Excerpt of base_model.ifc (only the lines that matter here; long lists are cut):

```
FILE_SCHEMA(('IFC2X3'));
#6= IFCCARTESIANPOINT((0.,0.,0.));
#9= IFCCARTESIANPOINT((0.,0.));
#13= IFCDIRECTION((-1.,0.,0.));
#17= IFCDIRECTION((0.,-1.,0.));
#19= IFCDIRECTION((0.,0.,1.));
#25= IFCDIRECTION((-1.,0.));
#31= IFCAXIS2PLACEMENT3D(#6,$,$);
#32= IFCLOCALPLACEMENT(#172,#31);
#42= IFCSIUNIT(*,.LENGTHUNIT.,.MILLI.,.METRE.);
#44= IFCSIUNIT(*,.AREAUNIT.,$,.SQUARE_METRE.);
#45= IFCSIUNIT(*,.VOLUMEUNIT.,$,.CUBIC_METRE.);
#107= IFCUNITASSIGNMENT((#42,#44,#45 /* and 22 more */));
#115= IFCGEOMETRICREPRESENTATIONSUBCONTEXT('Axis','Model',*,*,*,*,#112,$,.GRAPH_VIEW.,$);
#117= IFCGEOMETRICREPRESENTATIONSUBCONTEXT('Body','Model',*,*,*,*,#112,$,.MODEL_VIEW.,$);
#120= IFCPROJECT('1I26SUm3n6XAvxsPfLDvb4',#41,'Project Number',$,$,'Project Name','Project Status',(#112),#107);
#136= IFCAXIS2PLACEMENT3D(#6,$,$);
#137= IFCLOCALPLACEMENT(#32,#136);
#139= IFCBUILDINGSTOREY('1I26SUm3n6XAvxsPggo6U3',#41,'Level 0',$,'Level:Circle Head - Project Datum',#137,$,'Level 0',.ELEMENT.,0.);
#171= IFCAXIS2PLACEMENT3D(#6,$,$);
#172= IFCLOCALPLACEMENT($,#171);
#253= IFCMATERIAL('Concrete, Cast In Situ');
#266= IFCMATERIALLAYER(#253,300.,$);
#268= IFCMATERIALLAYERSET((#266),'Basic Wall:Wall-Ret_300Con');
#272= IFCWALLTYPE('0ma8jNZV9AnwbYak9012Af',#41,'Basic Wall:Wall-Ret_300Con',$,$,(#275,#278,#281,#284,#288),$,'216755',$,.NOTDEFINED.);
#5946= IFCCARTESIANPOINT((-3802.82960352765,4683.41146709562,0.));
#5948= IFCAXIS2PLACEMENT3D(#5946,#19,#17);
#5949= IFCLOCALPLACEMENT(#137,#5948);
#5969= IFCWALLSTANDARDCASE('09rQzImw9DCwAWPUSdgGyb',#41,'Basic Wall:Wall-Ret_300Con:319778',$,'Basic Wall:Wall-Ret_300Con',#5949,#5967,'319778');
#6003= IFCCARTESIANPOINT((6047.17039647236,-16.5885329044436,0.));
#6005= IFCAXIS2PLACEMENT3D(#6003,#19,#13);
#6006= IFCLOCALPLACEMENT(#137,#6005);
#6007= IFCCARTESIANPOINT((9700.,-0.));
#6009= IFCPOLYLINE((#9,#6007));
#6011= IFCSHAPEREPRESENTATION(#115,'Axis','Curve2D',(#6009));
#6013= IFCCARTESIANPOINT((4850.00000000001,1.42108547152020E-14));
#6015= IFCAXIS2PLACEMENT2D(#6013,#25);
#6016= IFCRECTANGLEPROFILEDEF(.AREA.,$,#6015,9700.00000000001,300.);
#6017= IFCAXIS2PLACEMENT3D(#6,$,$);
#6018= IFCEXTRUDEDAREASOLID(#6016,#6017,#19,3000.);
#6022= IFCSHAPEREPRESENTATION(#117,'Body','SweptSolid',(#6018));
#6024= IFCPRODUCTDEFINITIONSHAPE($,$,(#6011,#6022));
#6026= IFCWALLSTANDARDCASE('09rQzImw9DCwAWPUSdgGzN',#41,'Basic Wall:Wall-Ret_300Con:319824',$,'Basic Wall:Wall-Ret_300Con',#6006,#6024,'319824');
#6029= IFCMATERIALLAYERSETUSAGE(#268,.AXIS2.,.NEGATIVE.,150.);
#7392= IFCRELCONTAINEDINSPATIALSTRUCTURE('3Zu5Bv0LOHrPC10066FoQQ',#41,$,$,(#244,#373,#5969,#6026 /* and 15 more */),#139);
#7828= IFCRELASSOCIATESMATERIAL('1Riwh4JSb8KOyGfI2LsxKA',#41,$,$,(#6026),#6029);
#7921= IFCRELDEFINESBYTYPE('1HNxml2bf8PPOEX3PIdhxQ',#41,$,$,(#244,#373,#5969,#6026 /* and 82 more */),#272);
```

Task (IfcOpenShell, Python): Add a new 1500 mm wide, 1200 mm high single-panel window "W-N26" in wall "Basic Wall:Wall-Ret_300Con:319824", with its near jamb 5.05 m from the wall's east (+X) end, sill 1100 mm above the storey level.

```python
import numpy as np
import ifcopenshell
import ifcopenshell.api.feature
import ifcopenshell.api.geometry
import ifcopenshell.api.root
import ifcopenshell.api.spatial
import ifcopenshell.api.type
import ifcopenshell.geom
import ifcopenshell.util.element
import ifcopenshell.util.placement
import ifcopenshell.util.representation
import ifcopenshell.util.shape
import ifcopenshell.util.unit

model = ifcopenshell.open("base_model.ifc")
unit_scale = ifcopenshell.util.unit.calculate_unit_scale(model)
settings = ifcopenshell.geom.settings()


def volume(element):
    """Net volume in cubic metres, openings subtracted."""
    shape = ifcopenshell.geom.create_shape(settings, element)
    return ifcopenshell.util.shape.get_volume(shape.geometry)


wall = model.by_id(6026)
storey = ifcopenshell.util.element.get_container(wall, ifc_class="IfcBuildingStorey")
context = ifcopenshell.util.representation.get_context(model, "Model", "Body", "MODEL_VIEW")
before = volume(wall)

width, height, from_end, sill = 1.5, 1.2, 5.05, 1.1  # metres

# The wall runs along its own X axis, and the end named is its -X end.
wall_shape = ifcopenshell.geom.create_shape(settings, wall)
x, y, z = ifcopenshell.util.shape.get_vertices(wall_shape.geometry).T
start = x.min() + from_end
face, thickness = float(y.min()), float(y.max() - y.min())
wall_matrix = ifcopenshell.util.placement.get_local_placement(wall.ObjectPlacement)
level = ifcopenshell.util.placement.get_local_placement(storey.ObjectPlacement)[2, 3]


def in_wall(x, y):
    """Placement at x, y metres in the wall's axes, at sill height."""
    matrix = wall_matrix.copy()
    matrix[:, 3] = wall_matrix @ np.array([x / unit_scale, y / unit_scale, 0.0, 1.0])
    matrix[2, 3] = level + sill / unit_scale
    return matrix


# Opening: a box that overshoots both wall faces by 50 mm.
opening = ifcopenshell.api.root.create_entity(model, ifc_class="IfcOpeningElement")
box = ifcopenshell.api.geometry.add_wall_representation(
    model, context=context, length=width, height=height, thickness=thickness + 0.1
)
ifcopenshell.api.geometry.assign_representation(model, product=opening, representation=box)
ifcopenshell.api.geometry.edit_object_placement(model, product=opening, matrix=in_wall(start, face - 0.05), is_si=False)
ifcopenshell.api.feature.add_feature(model, feature=opening, element=wall)

window = ifcopenshell.api.root.create_entity(model, ifc_class="IfcWindow", name="W-N26")
window.OverallWidth, window.OverallHeight = width / unit_scale, height / unit_scale
body = ifcopenshell.api.geometry.add_window_representation(
    model,
    context=context,
    overall_width=window.OverallWidth,
    overall_height=window.OverallHeight,
    partition_type="SINGLE_PANEL",
)
ifcopenshell.api.geometry.assign_representation(model, product=window, representation=body)
ifcopenshell.api.spatial.assign_container(model, products=[window], relating_structure=storey)
fills = ifcopenshell.api.feature.add_filling(model, opening=opening, element=window)
fills.OwnerHistory = window.OwnerHistory  # required in IFC2X3

# IFC2X3 keeps the operation on the window style.
style = ifcopenshell.api.root.create_entity(model, ifc_class="IfcWindowStyle", name="W-N26")
style.OperationType, style.ConstructionType = "SINGLE_PANEL", "NOTDEFINED"
style.ParameterTakesPrecedence = style.Sizeable = False
ifcopenshell.api.type.assign_type(model, related_objects=[window], relating_type=style)

# Centre the window in the wall's thickness.
ifcopenshell.api.geometry.edit_object_placement(model, product=window, matrix=in_wall(start, face), is_si=False)
window_shape = ifcopenshell.geom.create_shape(settings, window)
depth = ifcopenshell.util.shape.get_vertices(window_shape.geometry)[:, 1]
offset = face + thickness / 2 - (depth.min() + depth.max()) / 2
ifcopenshell.api.geometry.edit_object_placement(model, product=window, matrix=in_wall(start, offset), is_si=False)

after = volume(wall)

print(f"wall volume {before:.3f} -> {after:.3f} m3")

model.write("base_model-out.ifc")
```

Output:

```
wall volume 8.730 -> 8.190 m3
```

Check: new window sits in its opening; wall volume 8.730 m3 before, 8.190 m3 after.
